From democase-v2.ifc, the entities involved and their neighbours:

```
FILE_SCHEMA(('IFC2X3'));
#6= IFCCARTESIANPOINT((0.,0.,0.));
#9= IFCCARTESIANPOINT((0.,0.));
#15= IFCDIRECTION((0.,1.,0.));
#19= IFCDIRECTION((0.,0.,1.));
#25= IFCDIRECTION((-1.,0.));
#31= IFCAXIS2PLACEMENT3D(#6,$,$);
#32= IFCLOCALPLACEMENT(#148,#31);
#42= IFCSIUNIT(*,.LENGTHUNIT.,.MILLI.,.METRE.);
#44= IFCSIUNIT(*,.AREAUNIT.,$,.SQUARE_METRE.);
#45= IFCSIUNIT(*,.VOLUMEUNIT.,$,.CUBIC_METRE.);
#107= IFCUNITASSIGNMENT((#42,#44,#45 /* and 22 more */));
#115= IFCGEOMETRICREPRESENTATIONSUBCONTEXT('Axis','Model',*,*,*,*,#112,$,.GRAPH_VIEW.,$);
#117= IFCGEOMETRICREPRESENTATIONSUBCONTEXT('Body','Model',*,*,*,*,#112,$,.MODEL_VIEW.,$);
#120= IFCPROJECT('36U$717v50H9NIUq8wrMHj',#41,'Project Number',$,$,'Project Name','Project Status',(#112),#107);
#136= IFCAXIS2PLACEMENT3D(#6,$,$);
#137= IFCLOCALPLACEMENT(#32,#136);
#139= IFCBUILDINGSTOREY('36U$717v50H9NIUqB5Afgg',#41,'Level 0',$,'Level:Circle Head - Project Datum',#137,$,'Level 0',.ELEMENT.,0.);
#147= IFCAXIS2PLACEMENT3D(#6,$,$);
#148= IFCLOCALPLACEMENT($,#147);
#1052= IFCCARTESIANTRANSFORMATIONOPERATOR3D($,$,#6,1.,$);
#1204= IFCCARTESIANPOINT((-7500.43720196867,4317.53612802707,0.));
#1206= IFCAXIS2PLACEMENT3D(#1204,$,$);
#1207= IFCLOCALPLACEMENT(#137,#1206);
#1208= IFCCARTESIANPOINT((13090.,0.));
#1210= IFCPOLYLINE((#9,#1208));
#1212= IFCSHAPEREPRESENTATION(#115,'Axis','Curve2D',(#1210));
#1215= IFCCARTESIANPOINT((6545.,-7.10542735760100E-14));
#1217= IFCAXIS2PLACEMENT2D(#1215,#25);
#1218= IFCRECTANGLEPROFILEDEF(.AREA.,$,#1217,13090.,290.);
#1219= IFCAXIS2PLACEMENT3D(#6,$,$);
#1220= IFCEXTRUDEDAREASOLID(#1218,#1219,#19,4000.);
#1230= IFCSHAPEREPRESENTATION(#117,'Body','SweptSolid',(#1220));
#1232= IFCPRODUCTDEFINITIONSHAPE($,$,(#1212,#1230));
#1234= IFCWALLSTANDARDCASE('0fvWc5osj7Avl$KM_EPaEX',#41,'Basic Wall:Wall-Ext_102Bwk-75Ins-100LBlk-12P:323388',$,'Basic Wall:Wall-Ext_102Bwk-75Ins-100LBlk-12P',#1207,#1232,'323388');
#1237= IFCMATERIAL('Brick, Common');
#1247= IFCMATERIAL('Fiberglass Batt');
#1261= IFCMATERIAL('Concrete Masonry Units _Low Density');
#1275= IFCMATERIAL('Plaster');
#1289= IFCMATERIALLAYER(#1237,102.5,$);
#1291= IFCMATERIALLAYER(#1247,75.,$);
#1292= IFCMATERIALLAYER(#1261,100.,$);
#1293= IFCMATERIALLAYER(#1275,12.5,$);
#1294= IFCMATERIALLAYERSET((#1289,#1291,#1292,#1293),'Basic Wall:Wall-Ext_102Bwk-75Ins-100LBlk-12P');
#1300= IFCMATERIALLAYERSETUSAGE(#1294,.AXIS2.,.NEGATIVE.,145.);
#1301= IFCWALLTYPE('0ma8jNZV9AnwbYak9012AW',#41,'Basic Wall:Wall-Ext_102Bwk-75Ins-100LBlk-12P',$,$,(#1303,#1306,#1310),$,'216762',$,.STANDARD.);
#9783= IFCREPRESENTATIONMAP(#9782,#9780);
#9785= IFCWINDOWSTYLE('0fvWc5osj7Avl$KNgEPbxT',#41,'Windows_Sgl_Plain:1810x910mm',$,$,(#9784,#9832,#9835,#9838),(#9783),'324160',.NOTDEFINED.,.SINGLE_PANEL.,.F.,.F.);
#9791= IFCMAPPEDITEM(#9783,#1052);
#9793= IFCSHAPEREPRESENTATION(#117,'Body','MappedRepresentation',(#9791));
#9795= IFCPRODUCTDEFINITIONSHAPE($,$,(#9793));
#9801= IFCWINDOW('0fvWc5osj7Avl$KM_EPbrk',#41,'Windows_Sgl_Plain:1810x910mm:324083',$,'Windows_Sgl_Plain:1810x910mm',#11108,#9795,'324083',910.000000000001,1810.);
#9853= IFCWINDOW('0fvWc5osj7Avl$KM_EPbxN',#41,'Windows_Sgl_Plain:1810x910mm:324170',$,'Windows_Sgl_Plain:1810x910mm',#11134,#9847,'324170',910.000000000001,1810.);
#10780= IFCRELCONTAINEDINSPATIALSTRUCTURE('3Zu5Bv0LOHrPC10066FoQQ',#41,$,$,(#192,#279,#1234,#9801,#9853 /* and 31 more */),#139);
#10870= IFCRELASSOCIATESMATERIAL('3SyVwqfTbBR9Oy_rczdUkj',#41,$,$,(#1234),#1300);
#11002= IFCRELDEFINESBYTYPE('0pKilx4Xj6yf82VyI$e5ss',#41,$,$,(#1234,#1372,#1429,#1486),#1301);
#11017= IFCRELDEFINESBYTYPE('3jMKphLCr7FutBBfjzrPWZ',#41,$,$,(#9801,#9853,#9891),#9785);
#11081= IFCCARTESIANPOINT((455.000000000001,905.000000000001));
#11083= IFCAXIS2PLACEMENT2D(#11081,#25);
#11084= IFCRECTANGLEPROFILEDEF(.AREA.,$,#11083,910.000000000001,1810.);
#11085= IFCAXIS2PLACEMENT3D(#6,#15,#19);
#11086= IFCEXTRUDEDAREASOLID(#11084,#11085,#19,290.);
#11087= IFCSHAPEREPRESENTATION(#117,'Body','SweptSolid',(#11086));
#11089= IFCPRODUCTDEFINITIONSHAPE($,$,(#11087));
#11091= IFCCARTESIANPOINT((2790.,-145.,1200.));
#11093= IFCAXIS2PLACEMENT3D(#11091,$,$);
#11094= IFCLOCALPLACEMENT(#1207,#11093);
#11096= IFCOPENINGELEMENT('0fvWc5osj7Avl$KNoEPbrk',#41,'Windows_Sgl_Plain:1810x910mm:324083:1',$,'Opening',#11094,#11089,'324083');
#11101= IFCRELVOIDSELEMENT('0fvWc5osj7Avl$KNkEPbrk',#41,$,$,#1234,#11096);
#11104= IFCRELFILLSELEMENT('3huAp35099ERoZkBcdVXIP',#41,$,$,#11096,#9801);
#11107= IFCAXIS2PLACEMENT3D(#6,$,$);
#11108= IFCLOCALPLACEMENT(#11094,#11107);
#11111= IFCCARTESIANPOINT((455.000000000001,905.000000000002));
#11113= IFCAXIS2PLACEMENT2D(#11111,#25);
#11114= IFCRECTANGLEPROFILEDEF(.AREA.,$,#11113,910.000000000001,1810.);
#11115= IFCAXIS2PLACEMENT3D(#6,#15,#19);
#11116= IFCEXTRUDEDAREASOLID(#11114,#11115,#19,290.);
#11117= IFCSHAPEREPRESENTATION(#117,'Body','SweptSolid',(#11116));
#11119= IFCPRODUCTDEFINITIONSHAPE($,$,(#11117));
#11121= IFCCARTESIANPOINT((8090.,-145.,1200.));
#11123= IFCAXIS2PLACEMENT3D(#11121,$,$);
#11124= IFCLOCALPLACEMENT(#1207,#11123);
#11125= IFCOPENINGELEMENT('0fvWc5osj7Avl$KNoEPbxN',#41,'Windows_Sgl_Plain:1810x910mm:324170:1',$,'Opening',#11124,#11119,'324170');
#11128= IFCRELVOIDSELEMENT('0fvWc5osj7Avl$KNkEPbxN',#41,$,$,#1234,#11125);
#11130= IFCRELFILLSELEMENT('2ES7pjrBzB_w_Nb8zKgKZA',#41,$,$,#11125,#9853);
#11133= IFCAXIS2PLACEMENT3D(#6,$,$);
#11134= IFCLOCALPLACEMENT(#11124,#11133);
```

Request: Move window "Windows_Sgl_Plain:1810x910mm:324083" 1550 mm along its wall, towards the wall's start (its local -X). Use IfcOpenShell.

```python
import ifcopenshell
import ifcopenshell.api.geometry
import ifcopenshell.util.placement

model = ifcopenshell.open("democase-v2.ifc")

window = model.by_id(9801)
opening = window.FillsVoids[0].RelatingOpeningElement
wall = opening.VoidsElements[0].RelatingBuildingElement

wall_matrix = ifcopenshell.util.placement.get_local_placement(wall.ObjectPlacement)
shift = wall_matrix[:3, 0] * -1550.0
before = ifcopenshell.util.placement.get_local_placement(window.ObjectPlacement)[:3, 3].copy()

# The window is placed relative to its opening, so it follows when the opening moves.
matrix = ifcopenshell.util.placement.get_local_placement(opening.ObjectPlacement)
matrix[:3, 3] += shift
ifcopenshell.api.geometry.edit_object_placement(
    model, product=opening, matrix=matrix, is_si=False, should_transform_children=True
)

after = ifcopenshell.util.placement.get_local_placement(window.ObjectPlacement)[:3, 3]
print("window moved by", (after - before).round(3) + 0.0)

model.write("democase-v2_v2.ifc")
```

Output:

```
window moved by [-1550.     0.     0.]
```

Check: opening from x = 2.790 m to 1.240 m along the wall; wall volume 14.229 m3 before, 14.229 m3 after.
